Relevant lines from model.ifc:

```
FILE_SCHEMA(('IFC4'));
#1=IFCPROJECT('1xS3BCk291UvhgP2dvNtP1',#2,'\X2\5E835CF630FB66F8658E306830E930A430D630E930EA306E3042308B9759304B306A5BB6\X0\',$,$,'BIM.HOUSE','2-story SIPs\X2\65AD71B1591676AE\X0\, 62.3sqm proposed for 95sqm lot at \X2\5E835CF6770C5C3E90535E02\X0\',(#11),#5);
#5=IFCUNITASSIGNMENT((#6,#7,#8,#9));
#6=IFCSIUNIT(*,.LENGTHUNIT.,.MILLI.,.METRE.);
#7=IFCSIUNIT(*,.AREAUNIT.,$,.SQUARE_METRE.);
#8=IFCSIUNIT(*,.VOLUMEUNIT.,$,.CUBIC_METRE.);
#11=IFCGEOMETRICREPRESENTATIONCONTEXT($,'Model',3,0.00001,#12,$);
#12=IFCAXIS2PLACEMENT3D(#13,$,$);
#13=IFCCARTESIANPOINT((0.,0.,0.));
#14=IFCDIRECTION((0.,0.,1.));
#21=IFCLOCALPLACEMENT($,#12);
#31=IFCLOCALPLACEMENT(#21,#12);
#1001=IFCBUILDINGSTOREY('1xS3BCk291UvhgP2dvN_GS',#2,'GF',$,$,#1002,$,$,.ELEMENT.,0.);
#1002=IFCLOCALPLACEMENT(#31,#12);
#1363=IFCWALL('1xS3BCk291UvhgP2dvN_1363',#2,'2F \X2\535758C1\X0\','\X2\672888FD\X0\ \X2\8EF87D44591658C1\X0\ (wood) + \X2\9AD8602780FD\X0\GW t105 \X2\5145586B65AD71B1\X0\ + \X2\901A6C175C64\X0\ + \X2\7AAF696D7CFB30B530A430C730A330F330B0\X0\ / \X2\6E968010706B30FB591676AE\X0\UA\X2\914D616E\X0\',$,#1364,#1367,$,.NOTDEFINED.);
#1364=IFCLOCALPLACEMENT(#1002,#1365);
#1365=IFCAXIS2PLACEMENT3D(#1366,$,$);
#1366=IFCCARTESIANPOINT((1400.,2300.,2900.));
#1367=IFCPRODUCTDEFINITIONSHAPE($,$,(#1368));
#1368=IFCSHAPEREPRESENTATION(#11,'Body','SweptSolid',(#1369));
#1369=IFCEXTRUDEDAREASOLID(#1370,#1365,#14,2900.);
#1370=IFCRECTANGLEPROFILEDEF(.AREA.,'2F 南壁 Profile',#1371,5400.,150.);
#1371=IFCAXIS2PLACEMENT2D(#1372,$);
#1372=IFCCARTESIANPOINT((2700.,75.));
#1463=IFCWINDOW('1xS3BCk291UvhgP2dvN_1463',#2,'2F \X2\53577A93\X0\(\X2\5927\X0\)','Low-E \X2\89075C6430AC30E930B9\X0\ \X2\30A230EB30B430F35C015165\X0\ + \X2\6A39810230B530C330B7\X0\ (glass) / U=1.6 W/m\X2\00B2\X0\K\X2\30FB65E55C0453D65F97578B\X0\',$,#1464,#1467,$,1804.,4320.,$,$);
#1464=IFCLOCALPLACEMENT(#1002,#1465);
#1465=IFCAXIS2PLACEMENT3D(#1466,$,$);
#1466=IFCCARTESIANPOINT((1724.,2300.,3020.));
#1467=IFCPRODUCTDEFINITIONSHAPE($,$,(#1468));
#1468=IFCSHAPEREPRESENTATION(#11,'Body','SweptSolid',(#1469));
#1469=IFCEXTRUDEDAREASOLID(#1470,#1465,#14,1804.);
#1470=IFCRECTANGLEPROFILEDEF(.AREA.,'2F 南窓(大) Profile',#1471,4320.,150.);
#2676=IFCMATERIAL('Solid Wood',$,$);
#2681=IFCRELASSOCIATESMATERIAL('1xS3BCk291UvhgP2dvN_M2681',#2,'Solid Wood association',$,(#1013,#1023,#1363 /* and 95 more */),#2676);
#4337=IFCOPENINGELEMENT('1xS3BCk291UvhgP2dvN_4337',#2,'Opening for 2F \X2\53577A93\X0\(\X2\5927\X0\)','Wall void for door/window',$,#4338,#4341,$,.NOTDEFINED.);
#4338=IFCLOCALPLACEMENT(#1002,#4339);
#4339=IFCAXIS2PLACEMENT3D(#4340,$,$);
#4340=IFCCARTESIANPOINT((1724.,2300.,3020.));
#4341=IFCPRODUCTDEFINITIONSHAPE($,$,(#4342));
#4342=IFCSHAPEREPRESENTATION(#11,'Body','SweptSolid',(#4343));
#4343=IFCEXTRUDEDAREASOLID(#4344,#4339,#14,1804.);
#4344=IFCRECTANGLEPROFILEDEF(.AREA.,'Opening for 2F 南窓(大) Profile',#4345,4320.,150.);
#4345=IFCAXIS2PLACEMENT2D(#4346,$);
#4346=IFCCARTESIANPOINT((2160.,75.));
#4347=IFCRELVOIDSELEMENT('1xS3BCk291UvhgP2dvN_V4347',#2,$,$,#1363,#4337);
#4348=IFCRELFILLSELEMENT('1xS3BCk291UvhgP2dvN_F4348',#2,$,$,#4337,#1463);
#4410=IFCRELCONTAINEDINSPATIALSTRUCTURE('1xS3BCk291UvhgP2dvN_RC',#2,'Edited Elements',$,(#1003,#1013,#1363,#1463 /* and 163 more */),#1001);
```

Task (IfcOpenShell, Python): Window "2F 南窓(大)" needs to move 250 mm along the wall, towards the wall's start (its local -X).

```python
import ifcopenshell
import ifcopenshell.api.geometry
import ifcopenshell.util.placement
import ifcopenshell.util.unit

model = ifcopenshell.open("model.ifc")
unit_scale = ifcopenshell.util.unit.calculate_unit_scale(model)

window = model.by_guid("1xS3BCk291UvhgP2dvN_1463")
opening = window.FillsVoids[0].RelatingOpeningElement
wall = opening.VoidsElements[0].RelatingBuildingElement

wall_matrix = ifcopenshell.util.placement.get_local_placement(wall.ObjectPlacement)
shift = wall_matrix[:3, 0] * -0.25 / unit_scale
before = ifcopenshell.util.placement.get_local_placement(window.ObjectPlacement)[:3, 3].copy()

# The window is not placed relative to its opening, so move both.
for product in (opening, window):
    matrix = ifcopenshell.util.placement.get_local_placement(product.ObjectPlacement)
    matrix[:3, 3] += shift
    ifcopenshell.api.geometry.edit_object_placement(model, product=product, matrix=matrix, is_si=False)

after = ifcopenshell.util.placement.get_local_placement(window.ObjectPlacement)[:3, 3]
print("window moved by", (after - before).round(3) + 0.0)

model.write("model_rev.ifc")
```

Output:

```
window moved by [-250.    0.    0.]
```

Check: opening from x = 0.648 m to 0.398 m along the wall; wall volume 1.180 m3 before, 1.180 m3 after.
